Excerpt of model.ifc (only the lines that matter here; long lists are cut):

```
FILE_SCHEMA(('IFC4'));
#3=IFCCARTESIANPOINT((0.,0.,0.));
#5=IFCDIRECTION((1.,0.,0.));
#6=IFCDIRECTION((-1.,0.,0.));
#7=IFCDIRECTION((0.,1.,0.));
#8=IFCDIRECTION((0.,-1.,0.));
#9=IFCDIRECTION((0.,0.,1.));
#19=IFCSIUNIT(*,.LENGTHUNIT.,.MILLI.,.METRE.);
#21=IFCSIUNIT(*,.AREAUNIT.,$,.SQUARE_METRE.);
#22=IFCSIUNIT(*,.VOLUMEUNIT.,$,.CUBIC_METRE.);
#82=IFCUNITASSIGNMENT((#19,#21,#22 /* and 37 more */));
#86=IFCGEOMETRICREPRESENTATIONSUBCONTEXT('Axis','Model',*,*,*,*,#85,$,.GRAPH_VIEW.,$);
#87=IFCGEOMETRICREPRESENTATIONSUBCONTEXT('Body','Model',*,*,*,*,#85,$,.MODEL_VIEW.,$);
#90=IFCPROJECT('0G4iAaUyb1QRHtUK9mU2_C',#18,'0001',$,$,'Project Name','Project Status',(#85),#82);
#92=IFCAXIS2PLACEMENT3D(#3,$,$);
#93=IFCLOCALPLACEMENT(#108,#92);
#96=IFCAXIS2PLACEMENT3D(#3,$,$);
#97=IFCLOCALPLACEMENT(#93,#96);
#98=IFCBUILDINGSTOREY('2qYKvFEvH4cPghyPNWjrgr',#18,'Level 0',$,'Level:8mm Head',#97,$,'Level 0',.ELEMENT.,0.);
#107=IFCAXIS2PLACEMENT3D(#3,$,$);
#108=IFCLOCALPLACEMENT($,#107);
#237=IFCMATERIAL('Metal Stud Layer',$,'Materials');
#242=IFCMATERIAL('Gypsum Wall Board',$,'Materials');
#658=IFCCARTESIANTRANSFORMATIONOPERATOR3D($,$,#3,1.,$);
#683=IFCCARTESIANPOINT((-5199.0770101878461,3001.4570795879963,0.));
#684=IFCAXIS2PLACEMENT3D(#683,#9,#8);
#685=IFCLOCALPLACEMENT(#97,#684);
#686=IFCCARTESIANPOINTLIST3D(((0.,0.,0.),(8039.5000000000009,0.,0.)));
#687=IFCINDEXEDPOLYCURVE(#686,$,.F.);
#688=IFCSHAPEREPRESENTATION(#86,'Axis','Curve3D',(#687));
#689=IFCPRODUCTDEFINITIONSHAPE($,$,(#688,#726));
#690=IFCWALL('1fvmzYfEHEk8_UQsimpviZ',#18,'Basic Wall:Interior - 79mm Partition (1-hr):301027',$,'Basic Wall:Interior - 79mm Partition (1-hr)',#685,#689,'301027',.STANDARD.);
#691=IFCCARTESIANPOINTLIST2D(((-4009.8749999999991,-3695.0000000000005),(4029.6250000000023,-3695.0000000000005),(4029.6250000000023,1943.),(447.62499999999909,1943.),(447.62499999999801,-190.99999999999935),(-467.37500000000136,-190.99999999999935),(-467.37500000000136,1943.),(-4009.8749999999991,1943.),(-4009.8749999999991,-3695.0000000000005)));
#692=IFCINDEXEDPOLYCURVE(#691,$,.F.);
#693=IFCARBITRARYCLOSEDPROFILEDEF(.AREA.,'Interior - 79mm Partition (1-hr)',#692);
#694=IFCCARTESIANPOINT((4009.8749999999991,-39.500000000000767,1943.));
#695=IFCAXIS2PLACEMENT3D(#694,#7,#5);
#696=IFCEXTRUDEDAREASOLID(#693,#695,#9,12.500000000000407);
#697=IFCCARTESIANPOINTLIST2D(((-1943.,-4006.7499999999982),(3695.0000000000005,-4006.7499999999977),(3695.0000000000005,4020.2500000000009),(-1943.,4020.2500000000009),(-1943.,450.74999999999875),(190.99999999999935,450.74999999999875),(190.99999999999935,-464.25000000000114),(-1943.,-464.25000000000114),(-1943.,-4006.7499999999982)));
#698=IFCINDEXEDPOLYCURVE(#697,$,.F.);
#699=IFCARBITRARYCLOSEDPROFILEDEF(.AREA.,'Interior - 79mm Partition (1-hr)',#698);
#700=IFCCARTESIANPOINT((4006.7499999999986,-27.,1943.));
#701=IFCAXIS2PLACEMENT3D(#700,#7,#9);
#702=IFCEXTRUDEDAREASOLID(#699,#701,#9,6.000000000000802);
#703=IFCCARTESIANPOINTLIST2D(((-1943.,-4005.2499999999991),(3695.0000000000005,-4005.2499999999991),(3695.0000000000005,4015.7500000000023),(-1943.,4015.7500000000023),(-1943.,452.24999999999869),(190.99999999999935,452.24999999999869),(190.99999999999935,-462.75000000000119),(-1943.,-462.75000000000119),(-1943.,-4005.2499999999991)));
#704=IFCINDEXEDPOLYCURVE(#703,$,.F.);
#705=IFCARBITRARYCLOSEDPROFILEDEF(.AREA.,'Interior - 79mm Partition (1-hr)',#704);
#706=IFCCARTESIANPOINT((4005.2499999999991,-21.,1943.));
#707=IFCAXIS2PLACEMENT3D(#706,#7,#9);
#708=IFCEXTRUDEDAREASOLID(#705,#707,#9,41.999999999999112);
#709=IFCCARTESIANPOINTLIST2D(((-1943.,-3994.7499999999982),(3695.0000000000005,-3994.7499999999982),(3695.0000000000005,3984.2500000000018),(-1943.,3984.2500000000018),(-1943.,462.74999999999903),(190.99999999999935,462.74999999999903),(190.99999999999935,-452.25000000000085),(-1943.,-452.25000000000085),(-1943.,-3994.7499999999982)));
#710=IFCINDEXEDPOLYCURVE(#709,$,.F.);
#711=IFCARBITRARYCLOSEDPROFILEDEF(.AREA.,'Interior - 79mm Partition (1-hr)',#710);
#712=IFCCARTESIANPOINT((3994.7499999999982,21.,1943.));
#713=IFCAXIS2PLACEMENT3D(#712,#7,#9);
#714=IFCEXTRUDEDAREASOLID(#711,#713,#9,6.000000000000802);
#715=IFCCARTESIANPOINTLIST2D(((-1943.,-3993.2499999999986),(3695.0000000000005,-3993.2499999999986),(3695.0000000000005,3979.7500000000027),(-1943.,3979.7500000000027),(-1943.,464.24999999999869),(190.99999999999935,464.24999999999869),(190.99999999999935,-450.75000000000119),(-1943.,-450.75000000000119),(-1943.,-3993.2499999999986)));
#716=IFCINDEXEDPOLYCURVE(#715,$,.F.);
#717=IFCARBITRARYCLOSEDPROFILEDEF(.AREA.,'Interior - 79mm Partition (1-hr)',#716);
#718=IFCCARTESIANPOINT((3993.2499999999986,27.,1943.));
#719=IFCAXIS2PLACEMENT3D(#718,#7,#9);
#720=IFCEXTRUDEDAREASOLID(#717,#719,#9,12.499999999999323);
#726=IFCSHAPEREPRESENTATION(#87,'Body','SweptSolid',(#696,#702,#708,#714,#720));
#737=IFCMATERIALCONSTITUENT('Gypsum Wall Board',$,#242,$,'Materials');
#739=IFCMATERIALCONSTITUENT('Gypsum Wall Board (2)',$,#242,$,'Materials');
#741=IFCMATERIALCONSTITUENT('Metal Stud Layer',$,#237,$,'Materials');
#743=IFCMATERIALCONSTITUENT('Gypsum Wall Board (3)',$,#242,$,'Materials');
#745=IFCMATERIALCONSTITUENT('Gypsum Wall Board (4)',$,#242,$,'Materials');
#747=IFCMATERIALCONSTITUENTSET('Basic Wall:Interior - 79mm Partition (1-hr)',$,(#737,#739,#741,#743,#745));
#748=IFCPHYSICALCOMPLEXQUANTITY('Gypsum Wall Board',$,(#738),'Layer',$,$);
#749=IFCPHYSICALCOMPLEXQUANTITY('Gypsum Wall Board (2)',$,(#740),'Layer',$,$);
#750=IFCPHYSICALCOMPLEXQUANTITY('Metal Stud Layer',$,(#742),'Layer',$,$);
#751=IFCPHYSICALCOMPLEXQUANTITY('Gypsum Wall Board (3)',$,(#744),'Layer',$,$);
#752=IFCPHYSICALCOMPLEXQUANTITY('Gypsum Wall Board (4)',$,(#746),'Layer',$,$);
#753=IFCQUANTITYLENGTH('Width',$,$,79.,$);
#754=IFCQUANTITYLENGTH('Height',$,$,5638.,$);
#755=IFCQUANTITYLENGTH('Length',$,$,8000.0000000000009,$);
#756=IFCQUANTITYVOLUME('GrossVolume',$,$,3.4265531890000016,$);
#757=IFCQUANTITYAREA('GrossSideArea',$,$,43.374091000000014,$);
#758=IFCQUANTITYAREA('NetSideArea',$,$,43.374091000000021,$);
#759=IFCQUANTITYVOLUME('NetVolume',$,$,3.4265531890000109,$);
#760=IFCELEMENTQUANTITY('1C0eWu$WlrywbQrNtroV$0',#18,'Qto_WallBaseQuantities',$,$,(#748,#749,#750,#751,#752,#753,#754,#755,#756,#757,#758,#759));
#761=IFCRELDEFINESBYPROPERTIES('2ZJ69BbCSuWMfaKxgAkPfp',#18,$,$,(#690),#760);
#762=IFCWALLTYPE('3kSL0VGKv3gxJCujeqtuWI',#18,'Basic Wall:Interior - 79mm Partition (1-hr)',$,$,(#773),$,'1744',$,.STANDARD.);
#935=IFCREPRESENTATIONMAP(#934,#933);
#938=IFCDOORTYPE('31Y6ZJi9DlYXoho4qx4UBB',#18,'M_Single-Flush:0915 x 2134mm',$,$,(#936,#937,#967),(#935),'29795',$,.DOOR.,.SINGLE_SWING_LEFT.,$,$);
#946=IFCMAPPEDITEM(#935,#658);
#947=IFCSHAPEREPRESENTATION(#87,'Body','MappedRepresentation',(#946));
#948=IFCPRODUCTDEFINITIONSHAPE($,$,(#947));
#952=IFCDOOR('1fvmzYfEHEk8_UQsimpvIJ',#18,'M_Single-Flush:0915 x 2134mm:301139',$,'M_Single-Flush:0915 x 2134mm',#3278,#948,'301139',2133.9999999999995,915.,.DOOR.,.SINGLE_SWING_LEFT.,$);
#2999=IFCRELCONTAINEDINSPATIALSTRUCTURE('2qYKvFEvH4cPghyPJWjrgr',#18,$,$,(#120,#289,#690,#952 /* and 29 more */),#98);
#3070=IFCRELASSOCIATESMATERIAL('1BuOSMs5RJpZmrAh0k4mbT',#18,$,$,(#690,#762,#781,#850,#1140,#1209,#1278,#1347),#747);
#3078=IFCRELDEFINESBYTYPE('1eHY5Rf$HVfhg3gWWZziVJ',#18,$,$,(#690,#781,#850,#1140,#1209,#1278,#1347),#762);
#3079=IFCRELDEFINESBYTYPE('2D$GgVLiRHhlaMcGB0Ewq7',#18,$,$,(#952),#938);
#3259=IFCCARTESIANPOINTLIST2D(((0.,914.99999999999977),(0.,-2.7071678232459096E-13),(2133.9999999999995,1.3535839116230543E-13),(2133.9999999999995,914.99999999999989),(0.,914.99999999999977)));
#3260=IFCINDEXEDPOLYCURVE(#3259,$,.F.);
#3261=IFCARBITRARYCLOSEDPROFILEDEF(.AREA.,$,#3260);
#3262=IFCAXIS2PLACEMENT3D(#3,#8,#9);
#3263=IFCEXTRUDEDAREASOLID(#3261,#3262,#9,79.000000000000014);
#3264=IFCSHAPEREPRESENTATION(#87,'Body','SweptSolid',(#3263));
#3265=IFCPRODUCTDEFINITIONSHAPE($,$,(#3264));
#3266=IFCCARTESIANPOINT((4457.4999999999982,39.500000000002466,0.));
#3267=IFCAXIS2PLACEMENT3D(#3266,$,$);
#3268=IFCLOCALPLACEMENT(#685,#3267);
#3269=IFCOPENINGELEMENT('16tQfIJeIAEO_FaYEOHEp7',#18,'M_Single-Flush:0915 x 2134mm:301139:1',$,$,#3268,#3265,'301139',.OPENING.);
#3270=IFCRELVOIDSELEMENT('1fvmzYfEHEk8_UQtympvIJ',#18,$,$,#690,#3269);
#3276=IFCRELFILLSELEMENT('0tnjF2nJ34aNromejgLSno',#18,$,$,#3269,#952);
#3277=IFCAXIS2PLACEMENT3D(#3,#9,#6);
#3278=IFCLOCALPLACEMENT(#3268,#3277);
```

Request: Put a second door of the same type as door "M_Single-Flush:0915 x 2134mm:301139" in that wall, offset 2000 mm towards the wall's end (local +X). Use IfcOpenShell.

```python
import ifcopenshell
import ifcopenshell.api.feature
import ifcopenshell.api.geometry
import ifcopenshell.api.pset
import ifcopenshell.api.root
import ifcopenshell.geom
import ifcopenshell.util.element
import ifcopenshell.util.placement
import ifcopenshell.util.shape
import ifcopenshell.util.unit

model = ifcopenshell.open("model.ifc")
unit_scale = ifcopenshell.util.unit.calculate_unit_scale(model)
area_scale = ifcopenshell.util.unit.calculate_unit_scale(model, "AREAUNIT")
volume_scale = ifcopenshell.util.unit.calculate_unit_scale(model, "VOLUMEUNIT")
settings = ifcopenshell.geom.settings()


def volume(element):
    """Net volume in cubic metres, openings subtracted."""
    shape = ifcopenshell.geom.create_shape(settings, element)
    return ifcopenshell.util.shape.get_volume(shape.geometry)


def reuse_history(source, copy):
    """copy_class also copies each property set's owner history, people and application; keep the originals."""
    for rel in copy.IsDefinedBy:
        if rel.is_a("IfcRelDefinesByProperties") and (history := rel.RelatingPropertyDefinition.OwnerHistory):
            rel.RelatingPropertyDefinition.OwnerHistory = source.OwnerHistory
            ifcopenshell.util.element.remove_deep2(model, history)


door = model.by_id(952)
opening = door.FillsVoids[0].RelatingOpeningElement
wall = opening.VoidsElements[0].RelatingBuildingElement
before = volume(wall)
shift = ifcopenshell.util.placement.get_local_placement(wall.ObjectPlacement)[:3, 0] * 2 / unit_scale

# copy_class copies the void relationship, type, container and properties, but no geometry.
new_opening = ifcopenshell.api.root.copy_class(model, product=opening)
new_opening.Representation = ifcopenshell.util.element.copy_deep(
    model, opening.Representation, exclude=["IfcGeometricRepresentationContext", "IfcRepresentationMap"]
)
new_opening.Name = "M_Single-Flush:0915 x 2134mm"
new_opening.Tag = None
reuse_history(opening, new_opening)
new_door = ifcopenshell.api.root.copy_class(model, product=door)
new_door.Representation = ifcopenshell.util.element.copy_deep(
    model, door.Representation, exclude=["IfcGeometricRepresentationContext", "IfcRepresentationMap"]
)
new_door.Name = "M_Single-Flush:0915 x 2134mm"
new_door.Tag = None
reuse_history(door, new_door)
ifcopenshell.api.feature.add_filling(model, opening=new_opening, element=new_door)

for old, new in ((opening, new_opening), (door, new_door)):
    matrix = ifcopenshell.util.placement.get_local_placement(old.ObjectPlacement)
    matrix[:3, 3] += shift
    ifcopenshell.api.geometry.edit_object_placement(model, product=new, matrix=matrix, is_si=False)

after = volume(wall)
thickness = 0.079  # wall thickness in metres

# Update the wall's stored quantities.
qto = model.by_id(ifcopenshell.util.element.get_pset(wall, "Qto_WallBaseQuantities", should_inherit=False)["id"])
ifcopenshell.api.pset.edit_qto(model, qto=qto, properties={
    "NetSideArea": after / thickness / area_scale,
    "NetVolume": after / volume_scale,
})

print(f"wall volume {before:.3f} -> {after:.3f} m3")

model.write("model-out.ifc")
```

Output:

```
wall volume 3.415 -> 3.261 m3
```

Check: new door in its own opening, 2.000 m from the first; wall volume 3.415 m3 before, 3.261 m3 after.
